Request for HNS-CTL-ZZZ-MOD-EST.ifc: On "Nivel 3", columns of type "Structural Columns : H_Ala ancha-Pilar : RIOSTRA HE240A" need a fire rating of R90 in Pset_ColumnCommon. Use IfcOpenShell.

First a look at what the model holds.

```python
import ifcopenshell
import ifcopenshell.util.element

model = ifcopenshell.open("HNS-CTL-ZZZ-MOD-EST.ifc")
print(model.schema)
storey = next(s for s in model.by_type("IfcBuildingStorey") if s.Name == "Nivel 3")
columns = [e for e in ifcopenshell.util.element.get_decomposition(storey) if e.is_a("IfcColumn")]
seen = {}
for e in columns:
    element_type = ifcopenshell.util.element.get_type(e)
    key = (element_type.Name if element_type != e and element_type else None, ifcopenshell.util.element.get_pset(e, "Pset_ColumnCommon", "FireRating"))
    seen[key] = seen.get(key, 0) + 1
for (name, value), count in sorted(seen.items(), key=str):
    print(count, "x", name, "|", value)
```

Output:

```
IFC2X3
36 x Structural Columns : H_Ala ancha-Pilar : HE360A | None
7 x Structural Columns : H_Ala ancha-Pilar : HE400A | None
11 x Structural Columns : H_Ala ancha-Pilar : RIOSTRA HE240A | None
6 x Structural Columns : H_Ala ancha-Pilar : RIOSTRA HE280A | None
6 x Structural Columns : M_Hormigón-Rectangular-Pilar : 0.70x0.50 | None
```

```python
import ifcopenshell
import ifcopenshell.api.pset
import ifcopenshell.util.element

model = ifcopenshell.open("HNS-CTL-ZZZ-MOD-EST.ifc")

storey = next(s for s in model.by_type("IfcBuildingStorey") if s.Name == "Nivel 3")
columns = [e for e in ifcopenshell.util.element.get_decomposition(storey) if e.is_a("IfcColumn")]

count = 0
for e in columns:
    element_type = ifcopenshell.util.element.get_type(e)
    if element_type in (None, e) or element_type.Name != "Structural Columns : H_Ala ancha-Pilar : RIOSTRA HE240A":
        continue
    # add_pset returns the element's existing set when there is one.
    pset = ifcopenshell.api.pset.add_pset(model, product=e, name="Pset_ColumnCommon")
    ifcopenshell.api.pset.edit_pset(model, pset=pset, properties={"FireRating": "R90"})
    count += 1

print(count, "columns updated")

model.write("HNS-CTL-ZZZ-MOD-EST_v2.ifc")
```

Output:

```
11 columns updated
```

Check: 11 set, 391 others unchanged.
